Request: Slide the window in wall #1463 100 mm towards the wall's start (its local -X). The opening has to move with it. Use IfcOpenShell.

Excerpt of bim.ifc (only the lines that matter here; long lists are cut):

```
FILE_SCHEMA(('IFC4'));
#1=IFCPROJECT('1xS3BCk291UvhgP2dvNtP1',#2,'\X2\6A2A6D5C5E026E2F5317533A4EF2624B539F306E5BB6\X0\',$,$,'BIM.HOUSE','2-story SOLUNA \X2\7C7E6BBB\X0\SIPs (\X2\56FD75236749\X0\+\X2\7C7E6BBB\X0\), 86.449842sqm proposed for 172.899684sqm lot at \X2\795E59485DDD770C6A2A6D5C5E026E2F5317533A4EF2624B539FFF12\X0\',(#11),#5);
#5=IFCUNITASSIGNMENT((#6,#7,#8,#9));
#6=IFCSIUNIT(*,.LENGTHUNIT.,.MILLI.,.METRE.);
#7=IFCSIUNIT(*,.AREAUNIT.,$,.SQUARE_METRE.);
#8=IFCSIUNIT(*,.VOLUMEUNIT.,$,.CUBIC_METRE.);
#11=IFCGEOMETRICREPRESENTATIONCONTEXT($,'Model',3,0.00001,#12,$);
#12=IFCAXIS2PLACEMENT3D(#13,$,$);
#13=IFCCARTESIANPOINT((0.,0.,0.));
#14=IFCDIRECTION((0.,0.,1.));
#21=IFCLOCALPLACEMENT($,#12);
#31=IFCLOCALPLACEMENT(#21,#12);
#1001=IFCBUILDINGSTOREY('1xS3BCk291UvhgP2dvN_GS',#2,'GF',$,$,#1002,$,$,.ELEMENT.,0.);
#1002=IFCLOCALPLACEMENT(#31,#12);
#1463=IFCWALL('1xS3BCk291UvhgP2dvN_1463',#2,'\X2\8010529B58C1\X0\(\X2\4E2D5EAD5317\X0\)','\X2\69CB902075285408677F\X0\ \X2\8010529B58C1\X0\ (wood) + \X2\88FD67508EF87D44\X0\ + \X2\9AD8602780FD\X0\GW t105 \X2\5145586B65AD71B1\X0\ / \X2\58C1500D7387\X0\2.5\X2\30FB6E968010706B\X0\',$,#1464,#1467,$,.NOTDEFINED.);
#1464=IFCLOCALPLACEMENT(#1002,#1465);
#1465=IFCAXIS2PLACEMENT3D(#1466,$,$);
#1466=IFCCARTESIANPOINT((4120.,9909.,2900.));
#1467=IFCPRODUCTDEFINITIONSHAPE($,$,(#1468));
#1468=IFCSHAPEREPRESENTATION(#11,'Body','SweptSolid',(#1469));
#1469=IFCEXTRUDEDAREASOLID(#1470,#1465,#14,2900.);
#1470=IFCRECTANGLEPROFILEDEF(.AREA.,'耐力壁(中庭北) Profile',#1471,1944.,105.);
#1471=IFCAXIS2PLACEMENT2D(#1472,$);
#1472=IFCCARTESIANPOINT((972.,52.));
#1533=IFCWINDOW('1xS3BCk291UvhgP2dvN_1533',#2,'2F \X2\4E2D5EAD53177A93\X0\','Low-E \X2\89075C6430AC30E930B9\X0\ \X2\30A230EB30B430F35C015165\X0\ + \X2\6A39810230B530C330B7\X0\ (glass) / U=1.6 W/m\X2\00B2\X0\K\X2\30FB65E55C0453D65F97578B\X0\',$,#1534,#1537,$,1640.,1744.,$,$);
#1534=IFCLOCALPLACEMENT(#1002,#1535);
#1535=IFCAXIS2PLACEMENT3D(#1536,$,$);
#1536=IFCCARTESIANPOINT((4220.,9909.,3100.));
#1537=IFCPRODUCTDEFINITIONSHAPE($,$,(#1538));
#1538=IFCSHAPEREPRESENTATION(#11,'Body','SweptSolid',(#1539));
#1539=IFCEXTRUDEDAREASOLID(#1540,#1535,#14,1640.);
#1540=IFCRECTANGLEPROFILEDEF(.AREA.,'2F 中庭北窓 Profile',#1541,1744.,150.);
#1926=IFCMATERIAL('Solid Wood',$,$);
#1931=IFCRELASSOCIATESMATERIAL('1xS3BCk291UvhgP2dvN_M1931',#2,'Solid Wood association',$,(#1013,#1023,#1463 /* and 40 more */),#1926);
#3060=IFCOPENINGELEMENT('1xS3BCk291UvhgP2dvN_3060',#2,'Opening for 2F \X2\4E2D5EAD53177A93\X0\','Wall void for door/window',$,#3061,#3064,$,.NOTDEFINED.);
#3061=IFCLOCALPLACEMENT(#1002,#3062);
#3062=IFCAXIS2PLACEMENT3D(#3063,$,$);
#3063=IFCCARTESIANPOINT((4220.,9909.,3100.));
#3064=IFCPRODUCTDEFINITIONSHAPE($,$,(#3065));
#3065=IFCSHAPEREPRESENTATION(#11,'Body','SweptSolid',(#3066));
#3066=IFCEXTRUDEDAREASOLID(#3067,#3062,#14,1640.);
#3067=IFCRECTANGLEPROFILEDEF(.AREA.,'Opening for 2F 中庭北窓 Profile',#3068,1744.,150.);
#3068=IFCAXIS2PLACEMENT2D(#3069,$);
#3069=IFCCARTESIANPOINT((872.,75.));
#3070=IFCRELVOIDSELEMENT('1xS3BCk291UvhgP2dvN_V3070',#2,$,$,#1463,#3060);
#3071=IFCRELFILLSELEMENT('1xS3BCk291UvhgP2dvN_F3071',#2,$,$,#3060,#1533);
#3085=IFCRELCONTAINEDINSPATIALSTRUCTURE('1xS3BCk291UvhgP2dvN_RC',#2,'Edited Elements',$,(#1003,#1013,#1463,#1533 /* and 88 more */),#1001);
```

```python
import ifcopenshell
import ifcopenshell.api.geometry
import ifcopenshell.util.placement

model = ifcopenshell.open("bim.ifc")

window = model.by_guid("1xS3BCk291UvhgP2dvN_1533")
opening = window.FillsVoids[0].RelatingOpeningElement
wall = opening.VoidsElements[0].RelatingBuildingElement

wall_matrix = ifcopenshell.util.placement.get_local_placement(wall.ObjectPlacement)
shift = wall_matrix[:3, 0] * -100.0
before = ifcopenshell.util.placement.get_local_placement(window.ObjectPlacement)[:3, 3].copy()

# The window is not placed relative to its opening, so move both.
for product in (opening, window):
    matrix = ifcopenshell.util.placement.get_local_placement(product.ObjectPlacement)
    matrix[:3, 3] += shift
    ifcopenshell.api.geometry.edit_object_placement(model, product=product, matrix=matrix, is_si=False)

after = ifcopenshell.util.placement.get_local_placement(window.ObjectPlacement)[:3, 3]
print("window moved by", (after - before).round(3) + 0.0)

model.write("bim_edited.ifc")
```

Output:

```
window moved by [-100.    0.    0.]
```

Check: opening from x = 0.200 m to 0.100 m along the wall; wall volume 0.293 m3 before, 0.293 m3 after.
